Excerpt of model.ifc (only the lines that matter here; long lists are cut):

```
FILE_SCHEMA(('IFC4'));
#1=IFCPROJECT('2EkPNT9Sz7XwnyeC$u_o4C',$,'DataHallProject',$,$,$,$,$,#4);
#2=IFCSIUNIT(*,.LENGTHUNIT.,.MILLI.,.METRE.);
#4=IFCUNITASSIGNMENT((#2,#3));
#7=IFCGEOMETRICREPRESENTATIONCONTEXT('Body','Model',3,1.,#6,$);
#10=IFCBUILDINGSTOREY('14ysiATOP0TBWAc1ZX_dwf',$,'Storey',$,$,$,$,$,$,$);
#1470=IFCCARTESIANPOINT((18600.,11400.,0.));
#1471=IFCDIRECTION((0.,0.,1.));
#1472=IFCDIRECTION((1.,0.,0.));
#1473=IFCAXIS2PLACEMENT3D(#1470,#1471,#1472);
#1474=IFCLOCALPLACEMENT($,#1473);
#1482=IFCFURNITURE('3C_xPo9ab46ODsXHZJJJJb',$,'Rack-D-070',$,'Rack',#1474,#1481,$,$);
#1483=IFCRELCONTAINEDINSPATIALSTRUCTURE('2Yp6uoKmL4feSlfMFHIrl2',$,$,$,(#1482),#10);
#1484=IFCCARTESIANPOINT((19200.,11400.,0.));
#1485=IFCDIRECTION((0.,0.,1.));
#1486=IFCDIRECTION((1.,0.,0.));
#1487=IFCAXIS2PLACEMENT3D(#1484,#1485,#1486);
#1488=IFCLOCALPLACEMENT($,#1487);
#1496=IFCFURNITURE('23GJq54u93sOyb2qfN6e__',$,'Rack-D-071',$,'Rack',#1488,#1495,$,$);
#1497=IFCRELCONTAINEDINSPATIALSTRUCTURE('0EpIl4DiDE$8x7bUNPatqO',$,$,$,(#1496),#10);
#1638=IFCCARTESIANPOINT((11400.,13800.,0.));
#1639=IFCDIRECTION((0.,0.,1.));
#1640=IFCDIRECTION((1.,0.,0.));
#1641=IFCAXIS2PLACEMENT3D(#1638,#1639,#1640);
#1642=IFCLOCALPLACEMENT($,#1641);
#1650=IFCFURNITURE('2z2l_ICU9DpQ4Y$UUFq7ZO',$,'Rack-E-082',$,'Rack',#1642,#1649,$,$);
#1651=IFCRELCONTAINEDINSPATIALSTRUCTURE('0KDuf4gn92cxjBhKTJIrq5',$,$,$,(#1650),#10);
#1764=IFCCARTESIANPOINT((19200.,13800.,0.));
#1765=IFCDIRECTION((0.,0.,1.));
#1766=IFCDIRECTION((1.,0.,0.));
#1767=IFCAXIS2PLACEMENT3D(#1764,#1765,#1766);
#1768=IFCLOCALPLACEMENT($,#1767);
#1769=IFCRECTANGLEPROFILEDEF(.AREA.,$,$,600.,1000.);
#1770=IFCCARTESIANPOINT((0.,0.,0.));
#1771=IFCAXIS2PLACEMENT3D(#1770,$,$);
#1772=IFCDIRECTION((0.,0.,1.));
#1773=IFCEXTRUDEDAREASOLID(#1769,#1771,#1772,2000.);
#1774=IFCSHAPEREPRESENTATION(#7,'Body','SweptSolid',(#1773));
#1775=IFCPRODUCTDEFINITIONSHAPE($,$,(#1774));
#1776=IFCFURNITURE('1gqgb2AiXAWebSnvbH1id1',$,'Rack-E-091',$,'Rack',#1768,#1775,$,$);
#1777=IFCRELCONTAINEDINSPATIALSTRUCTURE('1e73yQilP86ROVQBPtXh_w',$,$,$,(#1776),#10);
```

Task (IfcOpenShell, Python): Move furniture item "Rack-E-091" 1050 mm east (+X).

```python
import ifcopenshell
import ifcopenshell.api.geometry
import ifcopenshell.util.placement
import ifcopenshell.util.unit

model = ifcopenshell.open("model.ifc")
unit_scale = ifcopenshell.util.unit.calculate_unit_scale(model)

item = model.by_guid("1gqgb2AiXAWebSnvbH1id1")
matrix = ifcopenshell.util.placement.get_local_placement(item.ObjectPlacement)
matrix[0, 3] += 1.05 / unit_scale
ifcopenshell.api.geometry.edit_object_placement(model, product=item, matrix=matrix, is_si=False)

print(ifcopenshell.util.placement.get_local_placement(item.ObjectPlacement).round(3) + 0.0)

model.write("model_rev.ifc")
```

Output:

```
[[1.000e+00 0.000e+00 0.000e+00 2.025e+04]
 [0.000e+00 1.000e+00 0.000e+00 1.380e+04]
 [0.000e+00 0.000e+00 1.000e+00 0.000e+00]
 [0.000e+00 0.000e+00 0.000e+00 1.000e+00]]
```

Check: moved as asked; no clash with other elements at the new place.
